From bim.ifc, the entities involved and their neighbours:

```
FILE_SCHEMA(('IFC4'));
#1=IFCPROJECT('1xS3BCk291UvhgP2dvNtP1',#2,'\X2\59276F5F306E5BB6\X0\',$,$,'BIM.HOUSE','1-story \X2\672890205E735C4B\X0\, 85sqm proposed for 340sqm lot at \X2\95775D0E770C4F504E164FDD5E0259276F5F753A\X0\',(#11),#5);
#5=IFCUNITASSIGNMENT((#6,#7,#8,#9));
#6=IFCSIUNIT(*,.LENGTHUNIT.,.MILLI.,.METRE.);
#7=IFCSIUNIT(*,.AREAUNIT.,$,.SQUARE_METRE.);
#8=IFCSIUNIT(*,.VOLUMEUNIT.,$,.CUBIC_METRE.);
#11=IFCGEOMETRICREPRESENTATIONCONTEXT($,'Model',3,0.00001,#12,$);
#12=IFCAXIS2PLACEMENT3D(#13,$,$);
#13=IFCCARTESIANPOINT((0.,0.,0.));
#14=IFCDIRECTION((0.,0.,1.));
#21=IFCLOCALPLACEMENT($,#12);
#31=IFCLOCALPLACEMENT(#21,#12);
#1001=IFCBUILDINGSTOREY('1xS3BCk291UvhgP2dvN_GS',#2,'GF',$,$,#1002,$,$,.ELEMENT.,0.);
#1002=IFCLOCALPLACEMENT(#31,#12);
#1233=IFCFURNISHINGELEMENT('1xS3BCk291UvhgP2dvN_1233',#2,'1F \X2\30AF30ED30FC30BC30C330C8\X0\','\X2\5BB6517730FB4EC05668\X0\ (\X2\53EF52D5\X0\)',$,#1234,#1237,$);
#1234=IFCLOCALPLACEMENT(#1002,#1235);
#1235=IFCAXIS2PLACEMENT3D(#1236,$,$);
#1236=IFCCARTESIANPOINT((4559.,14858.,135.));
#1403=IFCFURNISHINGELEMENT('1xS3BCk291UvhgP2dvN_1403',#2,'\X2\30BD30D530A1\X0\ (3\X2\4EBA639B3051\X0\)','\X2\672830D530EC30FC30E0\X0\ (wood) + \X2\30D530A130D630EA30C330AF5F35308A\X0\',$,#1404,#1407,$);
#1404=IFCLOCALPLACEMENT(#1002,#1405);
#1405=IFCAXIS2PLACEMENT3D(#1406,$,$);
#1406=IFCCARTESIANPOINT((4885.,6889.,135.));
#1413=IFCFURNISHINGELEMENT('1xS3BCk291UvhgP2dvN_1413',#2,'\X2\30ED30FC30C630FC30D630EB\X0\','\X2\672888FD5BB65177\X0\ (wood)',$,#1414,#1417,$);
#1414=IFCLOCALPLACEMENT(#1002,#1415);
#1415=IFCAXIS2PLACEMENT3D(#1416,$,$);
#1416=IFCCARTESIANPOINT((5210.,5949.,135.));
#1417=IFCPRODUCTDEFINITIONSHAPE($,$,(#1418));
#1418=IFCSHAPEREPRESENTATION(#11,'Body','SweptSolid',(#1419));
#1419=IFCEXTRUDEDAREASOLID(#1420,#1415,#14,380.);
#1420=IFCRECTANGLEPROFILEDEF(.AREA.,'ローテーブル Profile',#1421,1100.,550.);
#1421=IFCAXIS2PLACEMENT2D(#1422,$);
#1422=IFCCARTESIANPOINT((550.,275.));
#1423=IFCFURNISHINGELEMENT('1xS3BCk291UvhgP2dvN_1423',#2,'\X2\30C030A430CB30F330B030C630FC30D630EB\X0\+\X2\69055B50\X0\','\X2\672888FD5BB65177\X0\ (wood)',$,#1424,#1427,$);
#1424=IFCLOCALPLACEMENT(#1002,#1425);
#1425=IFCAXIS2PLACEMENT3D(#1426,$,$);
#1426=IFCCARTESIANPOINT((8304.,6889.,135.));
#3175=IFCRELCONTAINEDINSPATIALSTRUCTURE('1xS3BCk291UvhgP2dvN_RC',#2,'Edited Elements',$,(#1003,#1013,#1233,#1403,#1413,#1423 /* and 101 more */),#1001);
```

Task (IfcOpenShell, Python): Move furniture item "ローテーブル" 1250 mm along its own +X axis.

```python
import ifcopenshell
import ifcopenshell.api.geometry
import ifcopenshell.util.placement
import ifcopenshell.util.unit

model = ifcopenshell.open("bim.ifc")
unit_scale = ifcopenshell.util.unit.calculate_unit_scale(model)

item = model.by_guid("1xS3BCk291UvhgP2dvN_1413")
matrix = ifcopenshell.util.placement.get_local_placement(item.ObjectPlacement)
matrix[:3, 3] += matrix[:3, 0] * 1.25 / unit_scale
ifcopenshell.api.geometry.edit_object_placement(model, product=item, matrix=matrix, is_si=False)

print(ifcopenshell.util.placement.get_local_placement(item.ObjectPlacement).round(3) + 0.0)

model.write("bim_edited.ifc")
```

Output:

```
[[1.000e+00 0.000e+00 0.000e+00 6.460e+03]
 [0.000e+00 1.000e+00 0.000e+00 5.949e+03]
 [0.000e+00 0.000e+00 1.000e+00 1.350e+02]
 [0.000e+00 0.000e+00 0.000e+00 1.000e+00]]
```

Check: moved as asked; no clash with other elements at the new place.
